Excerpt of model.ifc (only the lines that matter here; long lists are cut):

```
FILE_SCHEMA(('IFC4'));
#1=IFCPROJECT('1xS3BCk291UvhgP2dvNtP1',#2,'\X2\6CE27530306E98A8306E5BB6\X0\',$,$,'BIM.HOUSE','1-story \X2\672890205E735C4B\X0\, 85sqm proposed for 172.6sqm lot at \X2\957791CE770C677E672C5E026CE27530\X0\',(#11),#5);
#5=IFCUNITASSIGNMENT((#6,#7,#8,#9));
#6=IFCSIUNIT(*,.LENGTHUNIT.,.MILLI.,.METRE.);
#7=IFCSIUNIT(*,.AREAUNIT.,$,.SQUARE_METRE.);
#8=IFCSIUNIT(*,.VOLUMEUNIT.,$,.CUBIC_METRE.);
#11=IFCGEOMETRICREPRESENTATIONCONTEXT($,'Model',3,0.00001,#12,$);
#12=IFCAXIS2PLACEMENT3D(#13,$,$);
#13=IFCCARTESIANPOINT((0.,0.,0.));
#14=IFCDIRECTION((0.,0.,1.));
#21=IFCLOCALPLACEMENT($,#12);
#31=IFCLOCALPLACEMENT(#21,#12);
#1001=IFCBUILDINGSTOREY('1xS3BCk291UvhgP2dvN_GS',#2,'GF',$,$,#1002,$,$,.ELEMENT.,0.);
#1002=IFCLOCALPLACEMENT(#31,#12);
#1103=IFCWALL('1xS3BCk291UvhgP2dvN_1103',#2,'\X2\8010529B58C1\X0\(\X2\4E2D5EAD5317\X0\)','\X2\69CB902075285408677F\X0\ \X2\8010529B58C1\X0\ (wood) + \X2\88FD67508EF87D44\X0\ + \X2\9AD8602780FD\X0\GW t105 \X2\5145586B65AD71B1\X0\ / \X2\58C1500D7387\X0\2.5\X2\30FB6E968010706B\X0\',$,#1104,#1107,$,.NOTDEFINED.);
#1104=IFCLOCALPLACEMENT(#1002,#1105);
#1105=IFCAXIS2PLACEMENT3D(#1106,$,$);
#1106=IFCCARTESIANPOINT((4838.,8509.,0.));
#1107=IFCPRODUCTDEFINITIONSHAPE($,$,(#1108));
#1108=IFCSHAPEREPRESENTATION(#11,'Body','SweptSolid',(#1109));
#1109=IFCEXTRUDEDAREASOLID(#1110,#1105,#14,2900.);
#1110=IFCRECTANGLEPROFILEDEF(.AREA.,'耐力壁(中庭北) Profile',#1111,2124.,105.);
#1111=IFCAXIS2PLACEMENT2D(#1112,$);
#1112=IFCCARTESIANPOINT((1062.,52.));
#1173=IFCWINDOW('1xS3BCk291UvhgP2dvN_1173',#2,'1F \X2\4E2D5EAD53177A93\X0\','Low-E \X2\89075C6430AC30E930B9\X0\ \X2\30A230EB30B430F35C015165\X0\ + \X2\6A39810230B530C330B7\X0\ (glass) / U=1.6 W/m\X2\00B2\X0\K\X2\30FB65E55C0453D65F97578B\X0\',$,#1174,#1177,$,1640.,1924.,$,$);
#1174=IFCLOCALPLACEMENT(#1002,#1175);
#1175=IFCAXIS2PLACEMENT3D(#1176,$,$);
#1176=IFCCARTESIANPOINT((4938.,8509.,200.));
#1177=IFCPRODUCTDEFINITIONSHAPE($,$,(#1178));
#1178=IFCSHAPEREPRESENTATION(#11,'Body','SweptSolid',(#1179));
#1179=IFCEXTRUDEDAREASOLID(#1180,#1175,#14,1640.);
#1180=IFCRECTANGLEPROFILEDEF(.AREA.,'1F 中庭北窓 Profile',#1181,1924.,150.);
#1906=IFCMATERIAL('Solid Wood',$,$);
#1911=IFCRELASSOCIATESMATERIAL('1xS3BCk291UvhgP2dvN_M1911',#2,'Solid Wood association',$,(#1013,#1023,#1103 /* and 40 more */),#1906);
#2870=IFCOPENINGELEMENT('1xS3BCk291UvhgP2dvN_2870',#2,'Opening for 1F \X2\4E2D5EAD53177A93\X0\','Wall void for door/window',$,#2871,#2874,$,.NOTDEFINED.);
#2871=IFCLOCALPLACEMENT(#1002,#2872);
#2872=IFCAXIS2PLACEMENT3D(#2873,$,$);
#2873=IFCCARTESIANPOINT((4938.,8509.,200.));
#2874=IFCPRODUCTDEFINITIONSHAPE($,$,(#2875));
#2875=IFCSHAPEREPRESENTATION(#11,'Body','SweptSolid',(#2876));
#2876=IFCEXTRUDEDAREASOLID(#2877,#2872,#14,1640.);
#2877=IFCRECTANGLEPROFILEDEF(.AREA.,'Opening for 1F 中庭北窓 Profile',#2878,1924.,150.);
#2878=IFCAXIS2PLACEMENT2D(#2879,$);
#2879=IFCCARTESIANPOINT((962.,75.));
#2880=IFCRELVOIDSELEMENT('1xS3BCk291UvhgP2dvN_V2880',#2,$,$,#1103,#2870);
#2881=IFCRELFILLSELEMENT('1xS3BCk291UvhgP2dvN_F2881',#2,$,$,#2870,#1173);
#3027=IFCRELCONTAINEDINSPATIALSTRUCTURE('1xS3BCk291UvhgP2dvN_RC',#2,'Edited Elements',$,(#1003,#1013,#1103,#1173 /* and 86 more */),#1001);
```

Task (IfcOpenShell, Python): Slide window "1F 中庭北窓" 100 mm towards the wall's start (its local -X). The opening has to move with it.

```python
import ifcopenshell
import ifcopenshell.api.geometry
import ifcopenshell.util.placement

model = ifcopenshell.open("model.ifc")

window = model.by_guid("1xS3BCk291UvhgP2dvN_1173")
opening = window.FillsVoids[0].RelatingOpeningElement
wall = opening.VoidsElements[0].RelatingBuildingElement

wall_matrix = ifcopenshell.util.placement.get_local_placement(wall.ObjectPlacement)
shift = wall_matrix[:3, 0] * -100.0
before = ifcopenshell.util.placement.get_local_placement(window.ObjectPlacement)[:3, 3].copy()

# The window is not placed relative to its opening, so move both.
for product in (opening, window):
    matrix = ifcopenshell.util.placement.get_local_placement(product.ObjectPlacement)
    matrix[:3, 3] += shift
    ifcopenshell.api.geometry.edit_object_placement(model, product=product, matrix=matrix, is_si=False)

after = ifcopenshell.util.placement.get_local_placement(window.ObjectPlacement)[:3, 3]
print("window moved by", (after - before).round(3) + 0.0)

model.write("model_updated.ifc")
```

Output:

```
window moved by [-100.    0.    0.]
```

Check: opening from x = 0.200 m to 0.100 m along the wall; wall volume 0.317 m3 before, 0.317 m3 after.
